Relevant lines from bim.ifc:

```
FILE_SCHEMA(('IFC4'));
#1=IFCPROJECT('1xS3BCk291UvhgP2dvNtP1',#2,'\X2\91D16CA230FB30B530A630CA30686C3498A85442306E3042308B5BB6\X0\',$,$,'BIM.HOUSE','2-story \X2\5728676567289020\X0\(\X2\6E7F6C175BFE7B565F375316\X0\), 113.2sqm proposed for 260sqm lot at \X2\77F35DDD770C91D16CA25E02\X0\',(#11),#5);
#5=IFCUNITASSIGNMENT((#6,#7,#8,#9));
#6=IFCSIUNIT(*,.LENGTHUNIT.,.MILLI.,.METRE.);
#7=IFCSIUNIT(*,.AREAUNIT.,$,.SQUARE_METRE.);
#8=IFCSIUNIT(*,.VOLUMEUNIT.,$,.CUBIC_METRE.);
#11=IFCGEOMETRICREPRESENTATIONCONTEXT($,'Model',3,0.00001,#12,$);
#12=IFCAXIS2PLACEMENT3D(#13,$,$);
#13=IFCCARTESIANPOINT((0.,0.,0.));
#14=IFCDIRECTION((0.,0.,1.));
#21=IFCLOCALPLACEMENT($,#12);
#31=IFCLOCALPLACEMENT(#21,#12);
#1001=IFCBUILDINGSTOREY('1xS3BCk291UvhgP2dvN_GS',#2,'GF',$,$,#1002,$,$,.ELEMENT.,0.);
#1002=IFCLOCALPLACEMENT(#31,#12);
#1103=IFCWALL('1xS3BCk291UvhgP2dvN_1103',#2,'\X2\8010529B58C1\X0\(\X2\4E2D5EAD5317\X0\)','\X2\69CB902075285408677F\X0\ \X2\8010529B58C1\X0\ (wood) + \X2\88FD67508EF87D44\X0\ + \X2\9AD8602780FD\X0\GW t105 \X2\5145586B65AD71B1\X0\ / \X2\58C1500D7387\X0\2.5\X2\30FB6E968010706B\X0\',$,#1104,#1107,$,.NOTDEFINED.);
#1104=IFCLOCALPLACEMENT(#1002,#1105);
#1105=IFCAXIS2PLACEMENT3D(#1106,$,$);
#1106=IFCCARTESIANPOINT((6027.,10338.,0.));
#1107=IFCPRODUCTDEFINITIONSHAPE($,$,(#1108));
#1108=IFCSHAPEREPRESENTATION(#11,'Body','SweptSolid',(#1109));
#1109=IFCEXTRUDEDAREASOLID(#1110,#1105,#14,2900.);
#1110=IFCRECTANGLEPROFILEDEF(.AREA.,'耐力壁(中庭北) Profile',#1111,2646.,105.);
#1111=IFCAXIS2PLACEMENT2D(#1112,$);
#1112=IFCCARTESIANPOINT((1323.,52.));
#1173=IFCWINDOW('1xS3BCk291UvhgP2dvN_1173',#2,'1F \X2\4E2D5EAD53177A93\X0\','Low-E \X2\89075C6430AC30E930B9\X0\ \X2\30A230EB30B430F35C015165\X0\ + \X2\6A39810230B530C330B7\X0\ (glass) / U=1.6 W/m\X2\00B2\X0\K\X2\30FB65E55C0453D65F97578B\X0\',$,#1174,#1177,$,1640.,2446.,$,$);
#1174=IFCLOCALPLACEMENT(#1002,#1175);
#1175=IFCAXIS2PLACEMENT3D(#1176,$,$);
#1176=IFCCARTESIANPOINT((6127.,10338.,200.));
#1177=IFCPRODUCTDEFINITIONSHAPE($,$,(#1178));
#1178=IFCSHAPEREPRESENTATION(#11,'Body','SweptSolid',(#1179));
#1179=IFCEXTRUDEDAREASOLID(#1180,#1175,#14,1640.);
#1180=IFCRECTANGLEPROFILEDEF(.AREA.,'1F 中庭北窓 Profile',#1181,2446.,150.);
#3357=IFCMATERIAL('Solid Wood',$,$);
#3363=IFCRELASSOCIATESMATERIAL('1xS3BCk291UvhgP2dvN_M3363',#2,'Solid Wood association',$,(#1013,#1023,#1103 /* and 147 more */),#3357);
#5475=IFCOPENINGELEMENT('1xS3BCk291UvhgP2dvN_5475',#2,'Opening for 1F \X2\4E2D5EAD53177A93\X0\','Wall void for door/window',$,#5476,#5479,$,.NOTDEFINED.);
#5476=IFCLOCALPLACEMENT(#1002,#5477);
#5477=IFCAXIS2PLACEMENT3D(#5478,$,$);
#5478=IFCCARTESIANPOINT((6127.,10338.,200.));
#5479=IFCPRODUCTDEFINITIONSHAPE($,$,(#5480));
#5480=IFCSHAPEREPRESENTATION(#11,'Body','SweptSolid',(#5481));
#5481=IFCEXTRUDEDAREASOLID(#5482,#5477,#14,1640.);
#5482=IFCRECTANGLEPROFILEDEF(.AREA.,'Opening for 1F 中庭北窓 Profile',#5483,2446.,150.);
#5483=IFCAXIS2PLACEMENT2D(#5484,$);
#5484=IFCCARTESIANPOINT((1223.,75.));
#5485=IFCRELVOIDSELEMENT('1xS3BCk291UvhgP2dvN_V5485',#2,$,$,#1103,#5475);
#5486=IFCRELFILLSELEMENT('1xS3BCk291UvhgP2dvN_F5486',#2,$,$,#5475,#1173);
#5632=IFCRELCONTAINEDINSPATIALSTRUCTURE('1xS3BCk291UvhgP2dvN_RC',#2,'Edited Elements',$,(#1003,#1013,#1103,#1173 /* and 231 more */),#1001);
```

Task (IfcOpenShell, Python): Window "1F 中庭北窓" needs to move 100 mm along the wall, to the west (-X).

```python
import ifcopenshell
import ifcopenshell.api.geometry
import ifcopenshell.util.placement
import ifcopenshell.util.unit

model = ifcopenshell.open("bim.ifc")
unit_scale = ifcopenshell.util.unit.calculate_unit_scale(model)

window = model.by_guid("1xS3BCk291UvhgP2dvN_1173")
opening = window.FillsVoids[0].RelatingOpeningElement
wall = opening.VoidsElements[0].RelatingBuildingElement

wall_matrix = ifcopenshell.util.placement.get_local_placement(wall.ObjectPlacement)
shift = wall_matrix[:3, 0] * -0.1 / unit_scale
before = ifcopenshell.util.placement.get_local_placement(window.ObjectPlacement)[:3, 3].copy()

# The window is not placed relative to its opening, so move both.
for product in (opening, window):
    matrix = ifcopenshell.util.placement.get_local_placement(product.ObjectPlacement)
    matrix[:3, 3] += shift
    ifcopenshell.api.geometry.edit_object_placement(model, product=product, matrix=matrix, is_si=False)

after = ifcopenshell.util.placement.get_local_placement(window.ObjectPlacement)[:3, 3]
print("window moved by", (after - before).round(3) + 0.0)

model.write("bim_edited.ifc")
```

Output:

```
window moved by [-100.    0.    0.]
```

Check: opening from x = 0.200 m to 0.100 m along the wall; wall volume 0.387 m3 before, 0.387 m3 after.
